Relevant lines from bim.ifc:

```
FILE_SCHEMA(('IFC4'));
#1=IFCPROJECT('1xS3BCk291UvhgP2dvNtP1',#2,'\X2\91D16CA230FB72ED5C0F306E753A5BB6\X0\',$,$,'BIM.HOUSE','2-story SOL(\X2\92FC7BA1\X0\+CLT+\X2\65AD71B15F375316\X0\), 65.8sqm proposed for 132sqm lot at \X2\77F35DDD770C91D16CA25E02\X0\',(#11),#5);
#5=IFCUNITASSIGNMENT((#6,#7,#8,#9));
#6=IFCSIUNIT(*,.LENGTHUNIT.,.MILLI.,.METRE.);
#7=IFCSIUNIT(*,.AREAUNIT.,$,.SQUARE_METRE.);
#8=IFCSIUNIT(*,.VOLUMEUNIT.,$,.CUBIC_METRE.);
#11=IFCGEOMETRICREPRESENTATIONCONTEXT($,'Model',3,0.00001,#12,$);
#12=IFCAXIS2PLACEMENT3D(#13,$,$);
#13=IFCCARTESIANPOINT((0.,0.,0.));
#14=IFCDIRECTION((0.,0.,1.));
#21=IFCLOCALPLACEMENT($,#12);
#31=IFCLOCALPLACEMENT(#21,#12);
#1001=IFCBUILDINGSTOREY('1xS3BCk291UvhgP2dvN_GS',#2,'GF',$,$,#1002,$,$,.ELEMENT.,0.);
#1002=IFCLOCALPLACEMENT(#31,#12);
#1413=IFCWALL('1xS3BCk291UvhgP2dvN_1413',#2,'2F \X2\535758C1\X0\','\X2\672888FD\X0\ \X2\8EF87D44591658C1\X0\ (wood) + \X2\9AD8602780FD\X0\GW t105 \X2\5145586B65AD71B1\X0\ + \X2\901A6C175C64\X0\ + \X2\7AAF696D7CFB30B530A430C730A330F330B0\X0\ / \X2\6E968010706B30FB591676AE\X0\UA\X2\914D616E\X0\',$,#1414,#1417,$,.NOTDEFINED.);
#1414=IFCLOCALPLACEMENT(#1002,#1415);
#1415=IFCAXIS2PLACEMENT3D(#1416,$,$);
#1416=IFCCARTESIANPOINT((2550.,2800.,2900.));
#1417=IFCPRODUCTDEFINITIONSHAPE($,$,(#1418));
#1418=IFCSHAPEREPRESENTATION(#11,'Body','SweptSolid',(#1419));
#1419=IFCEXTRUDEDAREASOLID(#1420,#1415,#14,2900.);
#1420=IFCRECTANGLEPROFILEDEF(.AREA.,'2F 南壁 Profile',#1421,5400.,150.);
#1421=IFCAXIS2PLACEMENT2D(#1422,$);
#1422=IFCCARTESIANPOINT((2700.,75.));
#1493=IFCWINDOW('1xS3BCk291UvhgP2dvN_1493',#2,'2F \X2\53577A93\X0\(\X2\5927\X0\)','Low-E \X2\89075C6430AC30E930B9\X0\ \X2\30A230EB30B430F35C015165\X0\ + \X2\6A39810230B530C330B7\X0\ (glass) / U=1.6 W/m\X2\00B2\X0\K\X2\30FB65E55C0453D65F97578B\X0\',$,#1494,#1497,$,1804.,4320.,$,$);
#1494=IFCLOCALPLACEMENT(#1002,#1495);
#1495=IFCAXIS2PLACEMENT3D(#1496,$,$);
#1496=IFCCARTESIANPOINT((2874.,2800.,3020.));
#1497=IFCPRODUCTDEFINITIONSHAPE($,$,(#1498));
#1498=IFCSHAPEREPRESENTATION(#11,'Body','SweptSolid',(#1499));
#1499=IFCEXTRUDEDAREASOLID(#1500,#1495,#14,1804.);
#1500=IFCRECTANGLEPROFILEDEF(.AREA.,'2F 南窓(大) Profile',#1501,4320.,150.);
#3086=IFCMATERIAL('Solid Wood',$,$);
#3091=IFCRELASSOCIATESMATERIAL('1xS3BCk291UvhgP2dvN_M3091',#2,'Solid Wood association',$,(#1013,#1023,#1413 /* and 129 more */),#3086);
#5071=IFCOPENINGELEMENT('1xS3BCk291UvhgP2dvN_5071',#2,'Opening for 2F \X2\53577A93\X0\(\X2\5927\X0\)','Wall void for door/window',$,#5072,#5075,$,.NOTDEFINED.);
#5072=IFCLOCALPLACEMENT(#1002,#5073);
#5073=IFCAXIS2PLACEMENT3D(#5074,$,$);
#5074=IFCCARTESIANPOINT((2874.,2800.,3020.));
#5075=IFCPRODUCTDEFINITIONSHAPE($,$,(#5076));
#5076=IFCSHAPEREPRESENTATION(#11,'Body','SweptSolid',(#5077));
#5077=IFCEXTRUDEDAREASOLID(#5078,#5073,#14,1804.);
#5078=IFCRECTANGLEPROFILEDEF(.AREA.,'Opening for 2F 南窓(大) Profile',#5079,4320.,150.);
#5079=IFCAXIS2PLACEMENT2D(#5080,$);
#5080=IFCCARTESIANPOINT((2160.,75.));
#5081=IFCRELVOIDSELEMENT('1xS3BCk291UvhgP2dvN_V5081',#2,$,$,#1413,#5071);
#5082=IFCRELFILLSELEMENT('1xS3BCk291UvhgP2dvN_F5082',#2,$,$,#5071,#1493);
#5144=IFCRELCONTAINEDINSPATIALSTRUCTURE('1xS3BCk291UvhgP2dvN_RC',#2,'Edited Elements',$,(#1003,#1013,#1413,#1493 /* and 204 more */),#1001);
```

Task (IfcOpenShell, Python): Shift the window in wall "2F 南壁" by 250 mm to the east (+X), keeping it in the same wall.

```python
import ifcopenshell
import ifcopenshell.api.geometry
import ifcopenshell.util.placement
import ifcopenshell.util.unit

model = ifcopenshell.open("bim.ifc")
unit_scale = ifcopenshell.util.unit.calculate_unit_scale(model)

window = model.by_id(1493)
opening = window.FillsVoids[0].RelatingOpeningElement
wall = opening.VoidsElements[0].RelatingBuildingElement

wall_matrix = ifcopenshell.util.placement.get_local_placement(wall.ObjectPlacement)
shift = wall_matrix[:3, 0] * 0.25 / unit_scale
before = ifcopenshell.util.placement.get_local_placement(window.ObjectPlacement)[:3, 3].copy()

# The window is not placed relative to its opening, so move both.
for product in (opening, window):
    matrix = ifcopenshell.util.placement.get_local_placement(product.ObjectPlacement)
    matrix[:3, 3] += shift
    ifcopenshell.api.geometry.edit_object_placement(model, product=product, matrix=matrix, is_si=False)

after = ifcopenshell.util.placement.get_local_placement(window.ObjectPlacement)[:3, 3]
print("window moved by", (after - before).round(3) + 0.0)

model.write("bim_rev.ifc")
```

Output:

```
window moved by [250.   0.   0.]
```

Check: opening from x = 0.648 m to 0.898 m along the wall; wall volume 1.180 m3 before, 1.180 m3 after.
